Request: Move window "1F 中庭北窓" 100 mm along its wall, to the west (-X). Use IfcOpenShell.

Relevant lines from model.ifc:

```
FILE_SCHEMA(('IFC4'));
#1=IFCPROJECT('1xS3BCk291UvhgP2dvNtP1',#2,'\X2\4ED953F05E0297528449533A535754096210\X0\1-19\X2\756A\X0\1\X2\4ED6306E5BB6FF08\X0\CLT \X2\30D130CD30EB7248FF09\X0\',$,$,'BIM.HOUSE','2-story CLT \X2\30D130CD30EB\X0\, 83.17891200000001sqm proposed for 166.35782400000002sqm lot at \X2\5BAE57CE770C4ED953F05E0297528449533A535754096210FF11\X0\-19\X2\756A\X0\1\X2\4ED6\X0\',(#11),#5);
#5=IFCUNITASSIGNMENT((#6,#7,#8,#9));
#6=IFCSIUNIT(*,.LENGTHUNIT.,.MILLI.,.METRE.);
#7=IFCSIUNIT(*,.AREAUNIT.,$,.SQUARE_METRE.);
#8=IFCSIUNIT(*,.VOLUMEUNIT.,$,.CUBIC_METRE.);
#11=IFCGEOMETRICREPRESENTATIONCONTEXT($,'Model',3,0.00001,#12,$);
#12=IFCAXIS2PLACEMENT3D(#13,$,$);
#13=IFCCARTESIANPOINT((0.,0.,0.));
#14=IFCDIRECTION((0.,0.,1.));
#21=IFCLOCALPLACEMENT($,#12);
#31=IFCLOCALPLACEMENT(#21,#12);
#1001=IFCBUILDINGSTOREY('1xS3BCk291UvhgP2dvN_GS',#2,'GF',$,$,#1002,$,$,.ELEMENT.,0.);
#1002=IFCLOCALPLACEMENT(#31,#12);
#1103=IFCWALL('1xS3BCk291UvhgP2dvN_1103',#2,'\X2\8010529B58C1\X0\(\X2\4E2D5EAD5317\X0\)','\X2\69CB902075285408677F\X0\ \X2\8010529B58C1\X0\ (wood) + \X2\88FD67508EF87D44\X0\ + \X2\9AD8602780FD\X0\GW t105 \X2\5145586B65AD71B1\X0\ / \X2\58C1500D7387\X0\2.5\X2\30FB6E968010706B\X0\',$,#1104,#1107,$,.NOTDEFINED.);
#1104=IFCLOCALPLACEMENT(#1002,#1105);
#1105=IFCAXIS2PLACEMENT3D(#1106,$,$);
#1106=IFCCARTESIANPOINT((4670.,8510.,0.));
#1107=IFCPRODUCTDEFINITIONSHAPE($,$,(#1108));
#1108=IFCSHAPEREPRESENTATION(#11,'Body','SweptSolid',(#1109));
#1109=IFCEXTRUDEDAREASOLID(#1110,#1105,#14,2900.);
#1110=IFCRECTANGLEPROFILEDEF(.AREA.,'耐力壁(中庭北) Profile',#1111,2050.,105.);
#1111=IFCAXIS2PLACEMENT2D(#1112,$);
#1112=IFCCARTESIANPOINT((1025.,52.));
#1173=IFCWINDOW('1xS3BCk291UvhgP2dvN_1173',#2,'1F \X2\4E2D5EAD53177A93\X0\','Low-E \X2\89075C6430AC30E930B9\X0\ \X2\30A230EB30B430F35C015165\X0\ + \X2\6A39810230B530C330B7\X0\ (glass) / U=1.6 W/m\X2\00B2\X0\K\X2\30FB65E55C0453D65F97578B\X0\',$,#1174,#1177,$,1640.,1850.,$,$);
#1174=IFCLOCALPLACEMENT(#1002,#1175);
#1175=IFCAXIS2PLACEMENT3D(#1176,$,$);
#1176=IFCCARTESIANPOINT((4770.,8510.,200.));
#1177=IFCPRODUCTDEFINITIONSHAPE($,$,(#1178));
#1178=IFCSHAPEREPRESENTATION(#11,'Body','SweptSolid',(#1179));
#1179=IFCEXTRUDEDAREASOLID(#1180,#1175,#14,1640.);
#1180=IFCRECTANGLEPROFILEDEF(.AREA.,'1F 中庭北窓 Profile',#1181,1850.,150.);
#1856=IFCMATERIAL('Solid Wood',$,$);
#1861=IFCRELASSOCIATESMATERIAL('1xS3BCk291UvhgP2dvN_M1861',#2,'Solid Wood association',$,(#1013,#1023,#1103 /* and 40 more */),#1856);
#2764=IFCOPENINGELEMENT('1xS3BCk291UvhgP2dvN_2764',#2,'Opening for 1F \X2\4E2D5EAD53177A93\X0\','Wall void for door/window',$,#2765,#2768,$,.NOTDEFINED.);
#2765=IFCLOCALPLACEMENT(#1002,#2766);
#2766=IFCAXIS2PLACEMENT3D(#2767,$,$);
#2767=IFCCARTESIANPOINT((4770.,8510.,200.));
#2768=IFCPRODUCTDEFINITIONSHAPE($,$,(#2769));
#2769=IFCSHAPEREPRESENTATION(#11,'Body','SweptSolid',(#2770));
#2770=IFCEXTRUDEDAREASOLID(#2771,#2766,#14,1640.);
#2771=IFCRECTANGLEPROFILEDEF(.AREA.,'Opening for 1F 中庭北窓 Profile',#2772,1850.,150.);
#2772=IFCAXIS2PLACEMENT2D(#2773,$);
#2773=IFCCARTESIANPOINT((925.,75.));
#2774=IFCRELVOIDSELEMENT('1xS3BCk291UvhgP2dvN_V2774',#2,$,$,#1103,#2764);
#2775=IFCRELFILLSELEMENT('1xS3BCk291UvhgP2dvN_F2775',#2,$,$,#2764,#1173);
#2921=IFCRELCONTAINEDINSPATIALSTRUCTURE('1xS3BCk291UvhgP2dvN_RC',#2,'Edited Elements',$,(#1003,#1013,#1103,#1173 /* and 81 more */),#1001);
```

```python
import ifcopenshell
import ifcopenshell.api.geometry
import ifcopenshell.util.placement

model = ifcopenshell.open("model.ifc")

window = model.by_id(1173)
opening = window.FillsVoids[0].RelatingOpeningElement
wall = opening.VoidsElements[0].RelatingBuildingElement

wall_matrix = ifcopenshell.util.placement.get_local_placement(wall.ObjectPlacement)
shift = wall_matrix[:3, 0] * -100.0
before = ifcopenshell.util.placement.get_local_placement(window.ObjectPlacement)[:3, 3].copy()

# The window is not placed relative to its opening, so move both.
for product in (opening, window):
    matrix = ifcopenshell.util.placement.get_local_placement(product.ObjectPlacement)
    matrix[:3, 3] += shift
    ifcopenshell.api.geometry.edit_object_placement(model, product=product, matrix=matrix, is_si=False)

after = ifcopenshell.util.placement.get_local_placement(window.ObjectPlacement)[:3, 3]
print("window moved by", (after - before).round(3) + 0.0)

model.write("model_updated.ifc")
```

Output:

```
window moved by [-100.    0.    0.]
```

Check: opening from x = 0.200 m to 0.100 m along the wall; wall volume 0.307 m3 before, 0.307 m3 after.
